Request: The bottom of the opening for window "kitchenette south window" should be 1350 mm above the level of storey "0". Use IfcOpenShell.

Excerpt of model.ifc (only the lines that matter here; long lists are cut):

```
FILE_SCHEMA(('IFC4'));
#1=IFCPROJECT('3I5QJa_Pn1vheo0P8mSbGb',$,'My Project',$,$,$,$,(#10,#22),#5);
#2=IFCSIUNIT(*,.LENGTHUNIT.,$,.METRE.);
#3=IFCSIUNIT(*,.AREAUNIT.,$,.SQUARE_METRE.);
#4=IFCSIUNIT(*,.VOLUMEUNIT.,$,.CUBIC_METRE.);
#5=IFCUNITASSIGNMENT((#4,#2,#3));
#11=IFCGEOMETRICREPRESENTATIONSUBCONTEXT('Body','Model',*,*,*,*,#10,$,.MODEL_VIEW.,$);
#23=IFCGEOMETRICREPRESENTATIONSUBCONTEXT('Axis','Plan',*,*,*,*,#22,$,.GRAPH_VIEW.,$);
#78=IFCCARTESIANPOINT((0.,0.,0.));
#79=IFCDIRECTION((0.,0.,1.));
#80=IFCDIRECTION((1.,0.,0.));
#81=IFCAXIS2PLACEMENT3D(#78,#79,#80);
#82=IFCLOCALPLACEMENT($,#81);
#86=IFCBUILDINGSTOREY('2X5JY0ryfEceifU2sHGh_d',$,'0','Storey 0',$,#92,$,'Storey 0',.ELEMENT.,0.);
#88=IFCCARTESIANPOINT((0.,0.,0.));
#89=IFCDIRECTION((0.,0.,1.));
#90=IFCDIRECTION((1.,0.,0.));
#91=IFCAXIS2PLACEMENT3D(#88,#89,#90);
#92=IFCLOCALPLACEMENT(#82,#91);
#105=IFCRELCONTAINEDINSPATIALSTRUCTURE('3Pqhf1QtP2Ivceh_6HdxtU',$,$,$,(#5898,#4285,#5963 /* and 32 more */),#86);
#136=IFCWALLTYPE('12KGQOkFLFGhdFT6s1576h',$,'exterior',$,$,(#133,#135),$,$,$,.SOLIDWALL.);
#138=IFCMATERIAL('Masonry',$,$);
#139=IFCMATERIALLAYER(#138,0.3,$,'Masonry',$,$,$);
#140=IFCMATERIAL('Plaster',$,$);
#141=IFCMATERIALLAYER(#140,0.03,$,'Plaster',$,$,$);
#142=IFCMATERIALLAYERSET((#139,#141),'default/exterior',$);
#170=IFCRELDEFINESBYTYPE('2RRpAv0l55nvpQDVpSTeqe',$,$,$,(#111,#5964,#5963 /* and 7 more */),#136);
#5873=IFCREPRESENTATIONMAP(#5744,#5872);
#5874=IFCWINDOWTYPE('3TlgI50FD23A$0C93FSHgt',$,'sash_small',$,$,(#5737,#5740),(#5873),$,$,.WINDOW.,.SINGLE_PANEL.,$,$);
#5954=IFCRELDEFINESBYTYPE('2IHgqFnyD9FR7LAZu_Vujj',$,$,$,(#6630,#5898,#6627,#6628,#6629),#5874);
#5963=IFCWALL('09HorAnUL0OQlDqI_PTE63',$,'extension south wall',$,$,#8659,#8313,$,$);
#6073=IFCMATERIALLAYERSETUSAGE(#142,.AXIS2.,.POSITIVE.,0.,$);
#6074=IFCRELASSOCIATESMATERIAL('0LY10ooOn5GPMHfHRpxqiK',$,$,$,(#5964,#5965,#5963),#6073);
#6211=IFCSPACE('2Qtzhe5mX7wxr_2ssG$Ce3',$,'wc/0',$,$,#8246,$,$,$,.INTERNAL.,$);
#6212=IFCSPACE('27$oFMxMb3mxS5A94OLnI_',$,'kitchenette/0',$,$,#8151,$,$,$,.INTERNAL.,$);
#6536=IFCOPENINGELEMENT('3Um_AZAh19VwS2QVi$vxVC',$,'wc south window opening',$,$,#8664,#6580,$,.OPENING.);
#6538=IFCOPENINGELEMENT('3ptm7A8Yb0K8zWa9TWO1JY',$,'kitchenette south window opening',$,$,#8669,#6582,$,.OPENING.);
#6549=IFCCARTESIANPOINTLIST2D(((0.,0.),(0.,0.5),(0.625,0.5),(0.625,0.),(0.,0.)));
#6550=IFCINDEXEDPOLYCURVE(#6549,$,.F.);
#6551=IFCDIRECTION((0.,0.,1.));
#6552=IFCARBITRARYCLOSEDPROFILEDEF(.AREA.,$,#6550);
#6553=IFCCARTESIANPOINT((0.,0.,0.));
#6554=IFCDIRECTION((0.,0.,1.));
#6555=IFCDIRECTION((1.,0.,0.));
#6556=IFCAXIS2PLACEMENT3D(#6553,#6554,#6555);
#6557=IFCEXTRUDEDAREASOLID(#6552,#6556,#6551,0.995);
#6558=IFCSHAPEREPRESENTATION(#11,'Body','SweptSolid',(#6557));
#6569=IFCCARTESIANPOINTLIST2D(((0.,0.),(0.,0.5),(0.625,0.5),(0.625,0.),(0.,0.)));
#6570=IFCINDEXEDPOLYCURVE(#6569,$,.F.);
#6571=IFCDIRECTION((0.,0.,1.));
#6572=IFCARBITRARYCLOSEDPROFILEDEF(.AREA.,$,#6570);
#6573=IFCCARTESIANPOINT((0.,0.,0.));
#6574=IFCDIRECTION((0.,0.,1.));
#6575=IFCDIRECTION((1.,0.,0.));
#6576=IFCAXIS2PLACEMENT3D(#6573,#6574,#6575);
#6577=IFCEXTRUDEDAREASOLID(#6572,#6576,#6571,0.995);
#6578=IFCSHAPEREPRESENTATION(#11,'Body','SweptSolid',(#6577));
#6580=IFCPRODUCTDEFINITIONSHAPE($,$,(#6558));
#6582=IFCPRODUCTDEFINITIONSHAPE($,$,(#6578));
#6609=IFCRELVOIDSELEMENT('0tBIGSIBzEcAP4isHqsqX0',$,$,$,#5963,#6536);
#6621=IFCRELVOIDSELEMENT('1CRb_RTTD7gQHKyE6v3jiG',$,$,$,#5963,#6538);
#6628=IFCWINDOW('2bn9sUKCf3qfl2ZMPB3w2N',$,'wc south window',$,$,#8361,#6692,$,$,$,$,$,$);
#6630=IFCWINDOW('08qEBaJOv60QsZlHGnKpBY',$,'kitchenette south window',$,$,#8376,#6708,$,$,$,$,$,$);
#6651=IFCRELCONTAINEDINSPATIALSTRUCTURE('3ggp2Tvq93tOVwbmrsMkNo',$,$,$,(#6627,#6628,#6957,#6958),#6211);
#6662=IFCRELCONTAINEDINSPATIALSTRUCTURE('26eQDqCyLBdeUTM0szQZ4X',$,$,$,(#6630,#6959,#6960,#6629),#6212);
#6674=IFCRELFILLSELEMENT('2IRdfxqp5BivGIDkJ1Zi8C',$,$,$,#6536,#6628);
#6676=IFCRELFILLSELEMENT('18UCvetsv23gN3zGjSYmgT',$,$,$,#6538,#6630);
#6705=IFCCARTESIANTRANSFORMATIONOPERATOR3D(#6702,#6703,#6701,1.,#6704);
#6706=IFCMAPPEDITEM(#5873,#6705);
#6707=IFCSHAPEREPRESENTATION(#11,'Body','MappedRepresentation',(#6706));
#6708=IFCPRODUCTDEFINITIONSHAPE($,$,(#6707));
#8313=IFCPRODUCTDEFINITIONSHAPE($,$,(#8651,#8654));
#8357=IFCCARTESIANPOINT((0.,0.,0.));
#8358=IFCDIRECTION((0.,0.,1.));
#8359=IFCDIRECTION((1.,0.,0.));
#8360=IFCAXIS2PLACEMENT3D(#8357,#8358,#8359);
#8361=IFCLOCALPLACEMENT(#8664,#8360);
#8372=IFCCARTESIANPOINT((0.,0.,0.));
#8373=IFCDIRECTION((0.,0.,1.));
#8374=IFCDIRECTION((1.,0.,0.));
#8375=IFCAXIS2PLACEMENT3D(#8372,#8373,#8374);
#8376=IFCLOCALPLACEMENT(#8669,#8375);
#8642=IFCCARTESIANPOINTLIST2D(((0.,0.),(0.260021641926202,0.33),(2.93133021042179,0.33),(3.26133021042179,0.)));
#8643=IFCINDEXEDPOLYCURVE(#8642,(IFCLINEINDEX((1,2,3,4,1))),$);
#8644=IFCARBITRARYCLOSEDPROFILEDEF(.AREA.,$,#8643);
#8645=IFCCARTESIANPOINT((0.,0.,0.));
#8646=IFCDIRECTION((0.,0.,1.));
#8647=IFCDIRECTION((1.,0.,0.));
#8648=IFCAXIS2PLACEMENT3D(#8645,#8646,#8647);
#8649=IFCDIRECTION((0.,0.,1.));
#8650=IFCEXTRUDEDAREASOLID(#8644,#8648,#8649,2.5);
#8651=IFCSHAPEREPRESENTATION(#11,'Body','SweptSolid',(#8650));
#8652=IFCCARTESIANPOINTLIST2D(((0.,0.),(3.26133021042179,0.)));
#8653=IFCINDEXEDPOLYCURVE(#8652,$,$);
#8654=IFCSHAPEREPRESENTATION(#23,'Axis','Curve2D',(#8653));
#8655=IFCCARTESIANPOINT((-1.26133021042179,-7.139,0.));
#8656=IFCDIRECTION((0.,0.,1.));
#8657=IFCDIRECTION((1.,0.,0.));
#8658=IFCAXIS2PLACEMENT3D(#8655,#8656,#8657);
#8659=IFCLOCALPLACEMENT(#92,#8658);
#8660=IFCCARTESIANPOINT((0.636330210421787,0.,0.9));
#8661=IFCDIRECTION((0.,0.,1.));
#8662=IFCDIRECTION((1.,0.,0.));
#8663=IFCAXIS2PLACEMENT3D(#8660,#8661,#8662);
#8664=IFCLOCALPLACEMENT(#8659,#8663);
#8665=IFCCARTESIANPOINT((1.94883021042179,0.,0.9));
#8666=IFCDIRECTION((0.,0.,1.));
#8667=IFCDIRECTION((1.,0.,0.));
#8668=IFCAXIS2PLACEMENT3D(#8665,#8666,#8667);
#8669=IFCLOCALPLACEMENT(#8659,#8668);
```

```python
import numpy as np
import ifcopenshell
import ifcopenshell.api.geometry
import ifcopenshell.geom
import ifcopenshell.util.element
import ifcopenshell.util.placement
import ifcopenshell.util.shape
import ifcopenshell.util.unit

model = ifcopenshell.open("model.ifc")
unit_scale = ifcopenshell.util.unit.calculate_unit_scale(model)

window = model.by_guid("08qEBaJOv60QsZlHGnKpBY")
opening = window.FillsVoids[0].RelatingOpeningElement
storey = ifcopenshell.util.element.get_container(window, ifc_class="IfcBuildingStorey")
level = ifcopenshell.util.placement.get_local_placement(storey.ObjectPlacement)[2, 3]

# The opening's origin need not be at the sill, so measure its lowest point.
shape = ifcopenshell.geom.create_shape(ifcopenshell.geom.settings(), opening)
bottom = ifcopenshell.util.shape.get_shape_bottom_elevation(shape, shape.geometry) / unit_scale
dz = level + 1.35 / unit_scale - bottom

shift = np.array([0.0, 0.0, dz])
# The window is placed relative to its opening, so it follows when the opening moves.
matrix = ifcopenshell.util.placement.get_local_placement(opening.ObjectPlacement)
matrix[:3, 3] += shift
ifcopenshell.api.geometry.edit_object_placement(
    model, product=opening, matrix=matrix, is_si=False, should_transform_children=True
)

print(f"moved by {dz * unit_scale:+.3f} m")

model.write("model_rev.ifc")
```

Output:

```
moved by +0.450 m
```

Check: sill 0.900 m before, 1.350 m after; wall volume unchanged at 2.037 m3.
